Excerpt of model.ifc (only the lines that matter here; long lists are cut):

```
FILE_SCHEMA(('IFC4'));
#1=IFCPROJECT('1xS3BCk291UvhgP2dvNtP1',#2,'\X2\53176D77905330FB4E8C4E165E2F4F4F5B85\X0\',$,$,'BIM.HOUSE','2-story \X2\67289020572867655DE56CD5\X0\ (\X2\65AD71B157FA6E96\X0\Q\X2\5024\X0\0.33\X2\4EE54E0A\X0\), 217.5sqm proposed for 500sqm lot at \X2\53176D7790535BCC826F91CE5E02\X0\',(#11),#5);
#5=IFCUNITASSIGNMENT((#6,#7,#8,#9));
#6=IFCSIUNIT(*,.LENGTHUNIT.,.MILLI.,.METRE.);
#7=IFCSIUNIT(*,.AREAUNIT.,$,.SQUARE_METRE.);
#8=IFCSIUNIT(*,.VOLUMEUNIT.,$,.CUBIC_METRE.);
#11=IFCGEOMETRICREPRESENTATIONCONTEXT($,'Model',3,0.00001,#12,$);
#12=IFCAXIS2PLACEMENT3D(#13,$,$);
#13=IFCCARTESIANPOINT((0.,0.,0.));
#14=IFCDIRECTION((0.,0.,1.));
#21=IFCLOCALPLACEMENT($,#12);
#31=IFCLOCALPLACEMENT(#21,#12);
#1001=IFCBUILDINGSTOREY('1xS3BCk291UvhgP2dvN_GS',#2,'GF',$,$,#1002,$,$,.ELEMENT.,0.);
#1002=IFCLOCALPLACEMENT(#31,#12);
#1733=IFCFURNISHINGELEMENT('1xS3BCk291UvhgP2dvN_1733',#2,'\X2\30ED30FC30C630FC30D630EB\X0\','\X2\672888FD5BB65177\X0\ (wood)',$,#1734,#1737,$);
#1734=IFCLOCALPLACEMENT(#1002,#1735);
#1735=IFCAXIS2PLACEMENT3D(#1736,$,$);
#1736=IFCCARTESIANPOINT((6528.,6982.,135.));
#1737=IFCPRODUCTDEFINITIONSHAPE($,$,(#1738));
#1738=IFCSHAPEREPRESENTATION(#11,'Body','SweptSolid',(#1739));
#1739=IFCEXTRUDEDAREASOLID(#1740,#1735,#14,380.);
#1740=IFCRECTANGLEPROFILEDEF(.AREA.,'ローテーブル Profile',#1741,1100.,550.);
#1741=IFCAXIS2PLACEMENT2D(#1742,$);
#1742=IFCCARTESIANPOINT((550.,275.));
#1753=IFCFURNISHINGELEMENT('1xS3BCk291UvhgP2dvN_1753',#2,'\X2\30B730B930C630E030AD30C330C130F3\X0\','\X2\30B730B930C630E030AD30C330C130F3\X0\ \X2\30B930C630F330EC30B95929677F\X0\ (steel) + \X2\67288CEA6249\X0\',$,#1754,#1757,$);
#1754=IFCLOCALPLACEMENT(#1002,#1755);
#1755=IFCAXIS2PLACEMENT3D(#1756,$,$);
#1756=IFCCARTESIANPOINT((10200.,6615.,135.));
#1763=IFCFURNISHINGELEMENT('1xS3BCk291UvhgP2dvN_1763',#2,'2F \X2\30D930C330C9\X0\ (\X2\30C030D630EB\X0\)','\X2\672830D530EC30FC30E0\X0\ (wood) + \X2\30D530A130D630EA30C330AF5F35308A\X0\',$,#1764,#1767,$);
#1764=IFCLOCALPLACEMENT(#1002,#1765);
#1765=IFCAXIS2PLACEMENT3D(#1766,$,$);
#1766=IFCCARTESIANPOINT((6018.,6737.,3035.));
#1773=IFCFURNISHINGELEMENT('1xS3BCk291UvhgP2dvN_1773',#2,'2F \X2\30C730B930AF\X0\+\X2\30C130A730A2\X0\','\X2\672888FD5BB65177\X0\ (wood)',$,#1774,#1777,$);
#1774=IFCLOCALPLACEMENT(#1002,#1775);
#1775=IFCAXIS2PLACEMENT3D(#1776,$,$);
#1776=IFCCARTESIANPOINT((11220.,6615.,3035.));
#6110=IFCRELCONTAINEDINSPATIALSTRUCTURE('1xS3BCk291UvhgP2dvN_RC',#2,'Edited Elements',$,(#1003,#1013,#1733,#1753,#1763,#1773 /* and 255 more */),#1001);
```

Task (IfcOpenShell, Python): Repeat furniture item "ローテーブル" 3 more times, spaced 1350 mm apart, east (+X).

```python
import numpy as np
import ifcopenshell
import ifcopenshell.api.geometry
import ifcopenshell.api.root
import ifcopenshell.util.element
import ifcopenshell.util.placement
import ifcopenshell.util.unit

model = ifcopenshell.open("model.ifc")
unit_scale = ifcopenshell.util.unit.calculate_unit_scale(model)


def reuse_history(source, copy):
    """copy_class also copies each property set's owner history, people and application; keep the originals."""
    for rel in copy.IsDefinedBy:
        if rel.is_a("IfcRelDefinesByProperties") and (history := rel.RelatingPropertyDefinition.OwnerHistory):
            rel.RelatingPropertyDefinition.OwnerHistory = source.OwnerHistory
            ifcopenshell.util.element.remove_deep2(model, history)


source = model.by_guid("1xS3BCk291UvhgP2dvN_1733")
base = ifcopenshell.util.placement.get_local_placement(source.ObjectPlacement)
step = np.array([1.0, 0.0, 0.0]) * 1.35 / unit_scale

for i in range(1, 4):
    copy = ifcopenshell.api.root.copy_class(model, product=source)
    copy.Representation = ifcopenshell.util.element.copy_deep(
        model, source.Representation, exclude=["IfcGeometricRepresentationContext", "IfcRepresentationMap"]
    )
    reuse_history(source, copy)
    matrix = base.copy()
    matrix[:3, 3] += i * step
    print("added at", matrix[:3, 3].round(3) + 0.0)
    ifcopenshell.api.geometry.edit_object_placement(model, product=copy, matrix=matrix, is_si=False)

model.write("model_updated.ifc")
```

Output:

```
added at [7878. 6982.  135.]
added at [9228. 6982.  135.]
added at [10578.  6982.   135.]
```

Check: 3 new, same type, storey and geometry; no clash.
